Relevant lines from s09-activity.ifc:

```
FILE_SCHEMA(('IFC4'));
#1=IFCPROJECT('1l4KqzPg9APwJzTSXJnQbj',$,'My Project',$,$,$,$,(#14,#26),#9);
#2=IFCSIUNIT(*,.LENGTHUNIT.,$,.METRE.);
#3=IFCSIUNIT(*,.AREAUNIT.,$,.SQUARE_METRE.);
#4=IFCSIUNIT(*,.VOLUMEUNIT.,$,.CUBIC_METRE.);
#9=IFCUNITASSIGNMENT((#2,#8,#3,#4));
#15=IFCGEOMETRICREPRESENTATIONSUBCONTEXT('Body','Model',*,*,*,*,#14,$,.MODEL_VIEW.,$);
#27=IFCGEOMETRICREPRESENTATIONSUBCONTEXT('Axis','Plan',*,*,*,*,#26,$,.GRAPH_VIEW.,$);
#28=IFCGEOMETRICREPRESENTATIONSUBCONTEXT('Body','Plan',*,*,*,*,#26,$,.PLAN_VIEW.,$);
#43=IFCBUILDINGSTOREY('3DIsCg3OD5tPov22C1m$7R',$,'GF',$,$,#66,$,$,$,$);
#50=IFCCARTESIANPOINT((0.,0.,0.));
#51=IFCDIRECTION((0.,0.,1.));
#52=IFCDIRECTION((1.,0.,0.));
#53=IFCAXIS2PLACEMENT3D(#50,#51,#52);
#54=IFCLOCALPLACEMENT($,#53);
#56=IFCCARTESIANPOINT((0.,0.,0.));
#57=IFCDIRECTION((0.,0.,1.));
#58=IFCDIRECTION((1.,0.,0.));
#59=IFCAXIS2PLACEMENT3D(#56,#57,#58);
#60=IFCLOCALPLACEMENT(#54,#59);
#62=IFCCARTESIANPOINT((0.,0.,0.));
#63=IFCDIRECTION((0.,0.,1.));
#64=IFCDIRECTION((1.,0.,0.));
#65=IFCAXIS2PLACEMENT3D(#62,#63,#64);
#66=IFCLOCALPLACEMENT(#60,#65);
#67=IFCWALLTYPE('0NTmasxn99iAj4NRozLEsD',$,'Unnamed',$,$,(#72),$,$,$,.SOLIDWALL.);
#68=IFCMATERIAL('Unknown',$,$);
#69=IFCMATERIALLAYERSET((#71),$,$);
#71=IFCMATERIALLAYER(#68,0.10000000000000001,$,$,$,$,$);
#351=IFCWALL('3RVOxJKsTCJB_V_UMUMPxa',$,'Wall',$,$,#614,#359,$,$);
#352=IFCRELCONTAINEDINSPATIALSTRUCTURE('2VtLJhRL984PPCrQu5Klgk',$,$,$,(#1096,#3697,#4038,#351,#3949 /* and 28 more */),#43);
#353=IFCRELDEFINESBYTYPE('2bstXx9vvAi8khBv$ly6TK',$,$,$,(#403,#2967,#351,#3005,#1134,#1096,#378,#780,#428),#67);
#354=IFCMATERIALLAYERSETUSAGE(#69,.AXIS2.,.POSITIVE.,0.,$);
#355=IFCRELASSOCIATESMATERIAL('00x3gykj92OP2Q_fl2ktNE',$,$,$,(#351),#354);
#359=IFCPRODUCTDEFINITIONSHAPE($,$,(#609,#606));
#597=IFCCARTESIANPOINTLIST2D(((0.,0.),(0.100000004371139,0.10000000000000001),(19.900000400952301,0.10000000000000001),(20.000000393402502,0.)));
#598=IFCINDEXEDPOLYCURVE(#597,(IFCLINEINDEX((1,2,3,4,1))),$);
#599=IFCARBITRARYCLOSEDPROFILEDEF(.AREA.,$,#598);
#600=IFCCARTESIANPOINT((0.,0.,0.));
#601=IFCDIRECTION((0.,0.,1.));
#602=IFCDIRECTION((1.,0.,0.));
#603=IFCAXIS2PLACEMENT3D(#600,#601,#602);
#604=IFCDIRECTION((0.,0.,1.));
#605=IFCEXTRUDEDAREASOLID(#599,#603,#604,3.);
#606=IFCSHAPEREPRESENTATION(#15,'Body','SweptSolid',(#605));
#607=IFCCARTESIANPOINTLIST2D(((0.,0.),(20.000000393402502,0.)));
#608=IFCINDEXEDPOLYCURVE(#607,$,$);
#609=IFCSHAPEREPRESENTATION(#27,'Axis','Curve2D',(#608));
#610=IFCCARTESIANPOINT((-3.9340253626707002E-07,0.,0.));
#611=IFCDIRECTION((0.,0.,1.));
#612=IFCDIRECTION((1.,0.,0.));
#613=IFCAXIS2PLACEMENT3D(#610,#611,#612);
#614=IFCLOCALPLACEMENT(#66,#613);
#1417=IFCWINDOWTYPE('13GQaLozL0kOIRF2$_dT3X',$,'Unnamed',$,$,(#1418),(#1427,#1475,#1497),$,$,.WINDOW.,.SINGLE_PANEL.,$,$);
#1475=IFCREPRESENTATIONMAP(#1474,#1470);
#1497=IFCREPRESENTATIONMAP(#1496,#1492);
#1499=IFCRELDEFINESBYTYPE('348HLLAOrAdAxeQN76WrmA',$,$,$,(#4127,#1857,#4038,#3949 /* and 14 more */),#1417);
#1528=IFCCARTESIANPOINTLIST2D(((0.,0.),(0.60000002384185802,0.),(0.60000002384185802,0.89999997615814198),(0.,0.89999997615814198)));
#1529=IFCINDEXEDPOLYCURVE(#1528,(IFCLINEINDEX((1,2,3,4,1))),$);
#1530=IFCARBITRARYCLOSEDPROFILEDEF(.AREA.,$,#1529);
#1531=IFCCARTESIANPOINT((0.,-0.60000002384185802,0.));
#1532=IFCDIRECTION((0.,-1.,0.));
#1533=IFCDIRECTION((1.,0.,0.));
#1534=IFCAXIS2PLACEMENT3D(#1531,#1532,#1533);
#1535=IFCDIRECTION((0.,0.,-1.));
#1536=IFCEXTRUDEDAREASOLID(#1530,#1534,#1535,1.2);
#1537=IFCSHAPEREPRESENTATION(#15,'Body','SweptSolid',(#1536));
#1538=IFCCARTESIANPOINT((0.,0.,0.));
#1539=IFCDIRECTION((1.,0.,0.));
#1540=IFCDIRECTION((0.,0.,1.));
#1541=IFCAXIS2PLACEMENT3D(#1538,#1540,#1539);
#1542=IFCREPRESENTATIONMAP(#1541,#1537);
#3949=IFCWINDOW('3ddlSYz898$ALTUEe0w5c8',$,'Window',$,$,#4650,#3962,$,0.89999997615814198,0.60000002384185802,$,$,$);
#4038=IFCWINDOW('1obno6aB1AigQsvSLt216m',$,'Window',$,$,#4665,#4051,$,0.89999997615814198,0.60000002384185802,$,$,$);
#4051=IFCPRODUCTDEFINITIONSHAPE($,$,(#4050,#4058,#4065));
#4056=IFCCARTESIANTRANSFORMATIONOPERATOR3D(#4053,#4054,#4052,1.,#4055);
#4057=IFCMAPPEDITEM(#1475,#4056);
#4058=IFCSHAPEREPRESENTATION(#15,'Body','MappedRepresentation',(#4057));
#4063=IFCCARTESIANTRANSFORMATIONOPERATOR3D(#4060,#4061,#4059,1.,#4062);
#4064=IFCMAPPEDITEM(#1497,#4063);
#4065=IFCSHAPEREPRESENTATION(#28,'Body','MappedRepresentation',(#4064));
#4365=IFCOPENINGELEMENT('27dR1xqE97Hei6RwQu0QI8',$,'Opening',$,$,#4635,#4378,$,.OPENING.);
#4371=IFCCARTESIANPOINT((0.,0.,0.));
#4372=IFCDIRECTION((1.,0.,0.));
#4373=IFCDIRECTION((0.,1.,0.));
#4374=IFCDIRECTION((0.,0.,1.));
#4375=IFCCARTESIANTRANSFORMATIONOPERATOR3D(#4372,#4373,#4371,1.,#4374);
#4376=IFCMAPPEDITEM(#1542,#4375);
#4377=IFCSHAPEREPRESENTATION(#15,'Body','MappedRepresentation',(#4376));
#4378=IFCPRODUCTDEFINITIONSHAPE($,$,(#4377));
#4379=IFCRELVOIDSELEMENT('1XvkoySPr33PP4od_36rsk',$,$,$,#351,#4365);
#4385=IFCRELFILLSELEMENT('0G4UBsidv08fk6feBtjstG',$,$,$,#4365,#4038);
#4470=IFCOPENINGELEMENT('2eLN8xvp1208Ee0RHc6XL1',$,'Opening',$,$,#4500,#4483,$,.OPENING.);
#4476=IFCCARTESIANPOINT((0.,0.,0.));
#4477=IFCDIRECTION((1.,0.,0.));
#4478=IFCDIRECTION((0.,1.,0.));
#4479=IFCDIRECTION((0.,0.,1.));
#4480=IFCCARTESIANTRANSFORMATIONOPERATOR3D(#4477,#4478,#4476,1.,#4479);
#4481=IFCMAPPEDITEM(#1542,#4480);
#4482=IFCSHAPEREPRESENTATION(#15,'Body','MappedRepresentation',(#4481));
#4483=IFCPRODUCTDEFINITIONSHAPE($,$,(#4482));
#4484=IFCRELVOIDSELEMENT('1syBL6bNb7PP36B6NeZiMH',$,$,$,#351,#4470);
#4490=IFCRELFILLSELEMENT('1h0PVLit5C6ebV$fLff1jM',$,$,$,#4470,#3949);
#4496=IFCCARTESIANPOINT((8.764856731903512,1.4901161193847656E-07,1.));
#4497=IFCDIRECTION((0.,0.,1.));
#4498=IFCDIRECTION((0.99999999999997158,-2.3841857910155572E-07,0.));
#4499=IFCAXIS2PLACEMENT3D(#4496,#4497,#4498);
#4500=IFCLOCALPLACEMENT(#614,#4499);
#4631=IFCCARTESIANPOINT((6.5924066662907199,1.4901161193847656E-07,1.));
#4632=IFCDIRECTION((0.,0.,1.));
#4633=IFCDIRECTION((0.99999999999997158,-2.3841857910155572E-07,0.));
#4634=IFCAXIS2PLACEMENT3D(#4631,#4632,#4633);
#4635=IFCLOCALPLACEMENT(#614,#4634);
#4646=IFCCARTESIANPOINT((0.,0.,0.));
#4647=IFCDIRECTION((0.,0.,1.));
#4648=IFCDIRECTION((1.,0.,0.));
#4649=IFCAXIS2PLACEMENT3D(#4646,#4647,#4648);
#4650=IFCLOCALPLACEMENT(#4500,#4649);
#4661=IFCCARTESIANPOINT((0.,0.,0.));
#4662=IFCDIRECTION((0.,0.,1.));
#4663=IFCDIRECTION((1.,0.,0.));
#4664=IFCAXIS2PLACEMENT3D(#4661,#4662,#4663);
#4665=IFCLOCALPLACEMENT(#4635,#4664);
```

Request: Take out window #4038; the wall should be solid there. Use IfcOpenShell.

```python
import ifcopenshell
import ifcopenshell.api.feature
import ifcopenshell.api.root
import ifcopenshell.geom
import ifcopenshell.util.shape

model = ifcopenshell.open("s09-activity.ifc")
settings = ifcopenshell.geom.settings()


def volume(element):
    """Net volume in cubic metres, openings subtracted."""
    shape = ifcopenshell.geom.create_shape(settings, element)
    return ifcopenshell.util.shape.get_volume(shape.geometry)


window = model.by_guid("1obno6aB1AigQsvSLt216m")
opening = window.FillsVoids[0].RelatingOpeningElement
wall = opening.VoidsElements[0].RelatingBuildingElement
before = volume(wall)

ifcopenshell.api.root.remove_product(model, product=window)
ifcopenshell.api.feature.remove_feature(model, feature=opening)

after = volume(wall)

print(f"wall volume {before:.3f} -> {after:.3f} m3")

model.write("s09-activity_v2.ifc")
```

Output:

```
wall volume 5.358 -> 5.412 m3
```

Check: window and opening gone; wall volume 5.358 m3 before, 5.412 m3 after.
